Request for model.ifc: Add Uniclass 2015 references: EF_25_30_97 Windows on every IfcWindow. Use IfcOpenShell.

First a look at what the model holds.

```python
import ifcopenshell

model = ifcopenshell.open("model.ifc")
print(model.schema)
print("classifications:", [c.Name for c in model.by_type("IfcClassification")])
for ifc_class in ("IfcDoor", "IfcRoof", "IfcStair", "IfcWall", "IfcWindow"):
    print(ifc_class, len(model.by_type(ifc_class)))
```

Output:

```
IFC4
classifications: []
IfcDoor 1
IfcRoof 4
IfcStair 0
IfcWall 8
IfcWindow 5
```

```python
import ifcopenshell
import ifcopenshell.api.classification

model = ifcopenshell.open("model.ifc")

system = ifcopenshell.api.classification.add_classification(model, classification="Uniclass 2015")

codes = {
    "IfcWindow": ("EF_25_30_97", "Windows"),
}
for ifc_class, (code, name) in codes.items():
    products = model.by_type(ifc_class)
    ifcopenshell.api.classification.add_reference(
        model, products=products, classification=system, identification=code, name=name
    )
    print(code, len(products))

model.write("model_v2.ifc")
```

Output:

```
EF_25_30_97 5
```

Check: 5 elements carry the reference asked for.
